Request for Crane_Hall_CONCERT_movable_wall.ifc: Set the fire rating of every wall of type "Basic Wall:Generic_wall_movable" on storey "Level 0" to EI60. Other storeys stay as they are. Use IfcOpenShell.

First a look at what the model holds.

```python
import ifcopenshell
import ifcopenshell.util.element

model = ifcopenshell.open("Crane_Hall_CONCERT_movable_wall.ifc")
print(model.schema)
storey = next(s for s in model.by_type("IfcBuildingStorey") if s.Name == "Level 0")
walls = [e for e in ifcopenshell.util.element.get_decomposition(storey) if e.is_a("IfcWall")]
seen = {}
for e in walls:
    element_type = ifcopenshell.util.element.get_type(e)
    key = (element_type.Name if element_type != e and element_type else None, ifcopenshell.util.element.get_pset(e, "Pset_WallCommon", "FireRating"))
    seen[key] = seen.get(key, 0) + 1
for (name, value), count in sorted(seen.items(), key=str):
    print(count, "x", name, "|", value)
```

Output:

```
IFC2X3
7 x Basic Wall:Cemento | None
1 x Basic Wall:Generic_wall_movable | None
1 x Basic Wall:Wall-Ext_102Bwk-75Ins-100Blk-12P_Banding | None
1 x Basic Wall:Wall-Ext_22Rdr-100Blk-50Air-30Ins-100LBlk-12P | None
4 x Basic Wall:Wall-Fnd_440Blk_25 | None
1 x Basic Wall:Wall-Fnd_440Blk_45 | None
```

```python
import ifcopenshell
import ifcopenshell.api.pset
import ifcopenshell.util.element

model = ifcopenshell.open("Crane_Hall_CONCERT_movable_wall.ifc")

storey = next(s for s in model.by_type("IfcBuildingStorey") if s.Name == "Level 0")
walls = [e for e in ifcopenshell.util.element.get_decomposition(storey) if e.is_a("IfcWall")]

count = 0
for e in walls:
    element_type = ifcopenshell.util.element.get_type(e)
    if element_type in (None, e) or element_type.Name != "Basic Wall:Generic_wall_movable":
        continue
    # add_pset returns the element's existing set when there is one.
    pset = ifcopenshell.api.pset.add_pset(model, product=e, name="Pset_WallCommon")
    ifcopenshell.api.pset.edit_pset(model, pset=pset, properties={"FireRating": "EI60"})
    count += 1

print(count, "walls updated")

model.write("Crane_Hall_CONCERT_movable_wall_updated.ifc")
```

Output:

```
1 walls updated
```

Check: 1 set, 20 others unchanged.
